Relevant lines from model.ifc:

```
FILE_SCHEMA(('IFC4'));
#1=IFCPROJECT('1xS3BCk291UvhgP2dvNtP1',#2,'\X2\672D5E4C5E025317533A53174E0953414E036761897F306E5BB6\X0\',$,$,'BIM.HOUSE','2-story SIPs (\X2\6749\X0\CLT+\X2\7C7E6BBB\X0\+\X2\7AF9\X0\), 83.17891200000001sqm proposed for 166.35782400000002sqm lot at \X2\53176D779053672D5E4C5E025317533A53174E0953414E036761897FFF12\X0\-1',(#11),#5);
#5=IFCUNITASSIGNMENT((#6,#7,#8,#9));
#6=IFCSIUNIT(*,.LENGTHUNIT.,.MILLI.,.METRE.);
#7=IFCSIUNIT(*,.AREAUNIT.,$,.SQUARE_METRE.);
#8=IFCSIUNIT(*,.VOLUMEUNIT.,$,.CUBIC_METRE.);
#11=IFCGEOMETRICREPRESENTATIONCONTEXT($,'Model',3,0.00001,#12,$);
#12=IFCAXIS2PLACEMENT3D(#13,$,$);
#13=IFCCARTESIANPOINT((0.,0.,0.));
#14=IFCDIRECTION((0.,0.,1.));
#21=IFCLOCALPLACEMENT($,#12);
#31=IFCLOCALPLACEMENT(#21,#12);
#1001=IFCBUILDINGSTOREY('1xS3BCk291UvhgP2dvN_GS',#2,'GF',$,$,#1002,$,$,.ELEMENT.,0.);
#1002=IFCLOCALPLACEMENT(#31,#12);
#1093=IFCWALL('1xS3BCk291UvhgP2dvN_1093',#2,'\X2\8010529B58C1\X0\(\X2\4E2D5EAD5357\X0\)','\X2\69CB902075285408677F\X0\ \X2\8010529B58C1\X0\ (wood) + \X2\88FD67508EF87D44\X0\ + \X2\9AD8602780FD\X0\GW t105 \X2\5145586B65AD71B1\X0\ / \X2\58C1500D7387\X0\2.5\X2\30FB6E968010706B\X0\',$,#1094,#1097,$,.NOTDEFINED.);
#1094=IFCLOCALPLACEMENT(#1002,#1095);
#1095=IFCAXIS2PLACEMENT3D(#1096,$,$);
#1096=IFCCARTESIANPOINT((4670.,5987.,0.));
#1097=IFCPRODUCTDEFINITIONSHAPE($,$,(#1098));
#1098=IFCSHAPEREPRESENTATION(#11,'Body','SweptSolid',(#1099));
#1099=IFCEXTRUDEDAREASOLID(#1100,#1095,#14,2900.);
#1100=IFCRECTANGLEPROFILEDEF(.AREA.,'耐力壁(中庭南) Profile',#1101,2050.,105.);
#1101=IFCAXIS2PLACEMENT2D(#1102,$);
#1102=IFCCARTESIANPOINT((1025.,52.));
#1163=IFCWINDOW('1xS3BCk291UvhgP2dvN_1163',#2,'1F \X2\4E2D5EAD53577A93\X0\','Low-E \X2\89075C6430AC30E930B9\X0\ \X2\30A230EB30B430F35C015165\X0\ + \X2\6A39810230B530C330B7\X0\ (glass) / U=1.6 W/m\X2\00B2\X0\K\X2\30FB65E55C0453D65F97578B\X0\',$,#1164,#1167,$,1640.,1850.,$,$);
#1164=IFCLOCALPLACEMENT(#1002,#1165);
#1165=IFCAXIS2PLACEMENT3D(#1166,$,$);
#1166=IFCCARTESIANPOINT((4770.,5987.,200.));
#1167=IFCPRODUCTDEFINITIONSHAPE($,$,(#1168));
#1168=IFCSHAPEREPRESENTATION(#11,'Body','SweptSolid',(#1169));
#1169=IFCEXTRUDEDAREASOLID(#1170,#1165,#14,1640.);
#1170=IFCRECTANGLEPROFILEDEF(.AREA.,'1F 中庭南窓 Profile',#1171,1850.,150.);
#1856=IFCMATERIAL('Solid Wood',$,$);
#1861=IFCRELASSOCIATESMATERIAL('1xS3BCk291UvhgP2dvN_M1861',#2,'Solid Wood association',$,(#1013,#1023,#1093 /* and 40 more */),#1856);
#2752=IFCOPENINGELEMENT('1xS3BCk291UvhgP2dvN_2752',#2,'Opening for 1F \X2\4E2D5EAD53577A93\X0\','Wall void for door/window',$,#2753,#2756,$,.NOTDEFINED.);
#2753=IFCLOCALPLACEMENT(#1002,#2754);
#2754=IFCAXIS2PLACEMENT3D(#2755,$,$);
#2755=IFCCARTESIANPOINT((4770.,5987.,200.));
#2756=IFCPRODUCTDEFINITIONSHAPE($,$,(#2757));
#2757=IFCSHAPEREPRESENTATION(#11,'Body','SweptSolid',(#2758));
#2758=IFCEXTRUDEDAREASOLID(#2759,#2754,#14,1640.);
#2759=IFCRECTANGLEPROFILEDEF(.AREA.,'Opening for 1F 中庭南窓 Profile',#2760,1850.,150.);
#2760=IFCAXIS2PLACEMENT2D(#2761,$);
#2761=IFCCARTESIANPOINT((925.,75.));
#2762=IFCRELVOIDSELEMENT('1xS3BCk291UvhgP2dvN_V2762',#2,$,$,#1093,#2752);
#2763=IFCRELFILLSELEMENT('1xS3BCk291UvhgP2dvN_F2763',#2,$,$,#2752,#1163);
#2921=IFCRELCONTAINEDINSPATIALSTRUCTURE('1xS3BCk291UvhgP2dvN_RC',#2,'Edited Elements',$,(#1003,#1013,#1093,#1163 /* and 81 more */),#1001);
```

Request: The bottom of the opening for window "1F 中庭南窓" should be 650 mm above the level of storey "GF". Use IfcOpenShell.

```python
import numpy as np
import ifcopenshell
import ifcopenshell.api.geometry
import ifcopenshell.geom
import ifcopenshell.util.element
import ifcopenshell.util.placement
import ifcopenshell.util.shape
import ifcopenshell.util.unit

model = ifcopenshell.open("model.ifc")
unit_scale = ifcopenshell.util.unit.calculate_unit_scale(model)

window = model.by_guid("1xS3BCk291UvhgP2dvN_1163")
opening = window.FillsVoids[0].RelatingOpeningElement
storey = ifcopenshell.util.element.get_container(window, ifc_class="IfcBuildingStorey")
level = ifcopenshell.util.placement.get_local_placement(storey.ObjectPlacement)[2, 3]

# The opening's origin need not be at the sill, so measure its lowest point.
shape = ifcopenshell.geom.create_shape(ifcopenshell.geom.settings(), opening)
bottom = ifcopenshell.util.shape.get_shape_bottom_elevation(shape, shape.geometry) / unit_scale
dz = level + 0.65 / unit_scale - bottom

shift = np.array([0.0, 0.0, dz])
# The window is not placed relative to its opening, so move both.
for product in (opening, window):
    matrix = ifcopenshell.util.placement.get_local_placement(product.ObjectPlacement)
    matrix[:3, 3] += shift
    ifcopenshell.api.geometry.edit_object_placement(model, product=product, matrix=matrix, is_si=False)

print(f"moved by {dz * unit_scale:+.3f} m")

model.write("model_updated.ifc")
```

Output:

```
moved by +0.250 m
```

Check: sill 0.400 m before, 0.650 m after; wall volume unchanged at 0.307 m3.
